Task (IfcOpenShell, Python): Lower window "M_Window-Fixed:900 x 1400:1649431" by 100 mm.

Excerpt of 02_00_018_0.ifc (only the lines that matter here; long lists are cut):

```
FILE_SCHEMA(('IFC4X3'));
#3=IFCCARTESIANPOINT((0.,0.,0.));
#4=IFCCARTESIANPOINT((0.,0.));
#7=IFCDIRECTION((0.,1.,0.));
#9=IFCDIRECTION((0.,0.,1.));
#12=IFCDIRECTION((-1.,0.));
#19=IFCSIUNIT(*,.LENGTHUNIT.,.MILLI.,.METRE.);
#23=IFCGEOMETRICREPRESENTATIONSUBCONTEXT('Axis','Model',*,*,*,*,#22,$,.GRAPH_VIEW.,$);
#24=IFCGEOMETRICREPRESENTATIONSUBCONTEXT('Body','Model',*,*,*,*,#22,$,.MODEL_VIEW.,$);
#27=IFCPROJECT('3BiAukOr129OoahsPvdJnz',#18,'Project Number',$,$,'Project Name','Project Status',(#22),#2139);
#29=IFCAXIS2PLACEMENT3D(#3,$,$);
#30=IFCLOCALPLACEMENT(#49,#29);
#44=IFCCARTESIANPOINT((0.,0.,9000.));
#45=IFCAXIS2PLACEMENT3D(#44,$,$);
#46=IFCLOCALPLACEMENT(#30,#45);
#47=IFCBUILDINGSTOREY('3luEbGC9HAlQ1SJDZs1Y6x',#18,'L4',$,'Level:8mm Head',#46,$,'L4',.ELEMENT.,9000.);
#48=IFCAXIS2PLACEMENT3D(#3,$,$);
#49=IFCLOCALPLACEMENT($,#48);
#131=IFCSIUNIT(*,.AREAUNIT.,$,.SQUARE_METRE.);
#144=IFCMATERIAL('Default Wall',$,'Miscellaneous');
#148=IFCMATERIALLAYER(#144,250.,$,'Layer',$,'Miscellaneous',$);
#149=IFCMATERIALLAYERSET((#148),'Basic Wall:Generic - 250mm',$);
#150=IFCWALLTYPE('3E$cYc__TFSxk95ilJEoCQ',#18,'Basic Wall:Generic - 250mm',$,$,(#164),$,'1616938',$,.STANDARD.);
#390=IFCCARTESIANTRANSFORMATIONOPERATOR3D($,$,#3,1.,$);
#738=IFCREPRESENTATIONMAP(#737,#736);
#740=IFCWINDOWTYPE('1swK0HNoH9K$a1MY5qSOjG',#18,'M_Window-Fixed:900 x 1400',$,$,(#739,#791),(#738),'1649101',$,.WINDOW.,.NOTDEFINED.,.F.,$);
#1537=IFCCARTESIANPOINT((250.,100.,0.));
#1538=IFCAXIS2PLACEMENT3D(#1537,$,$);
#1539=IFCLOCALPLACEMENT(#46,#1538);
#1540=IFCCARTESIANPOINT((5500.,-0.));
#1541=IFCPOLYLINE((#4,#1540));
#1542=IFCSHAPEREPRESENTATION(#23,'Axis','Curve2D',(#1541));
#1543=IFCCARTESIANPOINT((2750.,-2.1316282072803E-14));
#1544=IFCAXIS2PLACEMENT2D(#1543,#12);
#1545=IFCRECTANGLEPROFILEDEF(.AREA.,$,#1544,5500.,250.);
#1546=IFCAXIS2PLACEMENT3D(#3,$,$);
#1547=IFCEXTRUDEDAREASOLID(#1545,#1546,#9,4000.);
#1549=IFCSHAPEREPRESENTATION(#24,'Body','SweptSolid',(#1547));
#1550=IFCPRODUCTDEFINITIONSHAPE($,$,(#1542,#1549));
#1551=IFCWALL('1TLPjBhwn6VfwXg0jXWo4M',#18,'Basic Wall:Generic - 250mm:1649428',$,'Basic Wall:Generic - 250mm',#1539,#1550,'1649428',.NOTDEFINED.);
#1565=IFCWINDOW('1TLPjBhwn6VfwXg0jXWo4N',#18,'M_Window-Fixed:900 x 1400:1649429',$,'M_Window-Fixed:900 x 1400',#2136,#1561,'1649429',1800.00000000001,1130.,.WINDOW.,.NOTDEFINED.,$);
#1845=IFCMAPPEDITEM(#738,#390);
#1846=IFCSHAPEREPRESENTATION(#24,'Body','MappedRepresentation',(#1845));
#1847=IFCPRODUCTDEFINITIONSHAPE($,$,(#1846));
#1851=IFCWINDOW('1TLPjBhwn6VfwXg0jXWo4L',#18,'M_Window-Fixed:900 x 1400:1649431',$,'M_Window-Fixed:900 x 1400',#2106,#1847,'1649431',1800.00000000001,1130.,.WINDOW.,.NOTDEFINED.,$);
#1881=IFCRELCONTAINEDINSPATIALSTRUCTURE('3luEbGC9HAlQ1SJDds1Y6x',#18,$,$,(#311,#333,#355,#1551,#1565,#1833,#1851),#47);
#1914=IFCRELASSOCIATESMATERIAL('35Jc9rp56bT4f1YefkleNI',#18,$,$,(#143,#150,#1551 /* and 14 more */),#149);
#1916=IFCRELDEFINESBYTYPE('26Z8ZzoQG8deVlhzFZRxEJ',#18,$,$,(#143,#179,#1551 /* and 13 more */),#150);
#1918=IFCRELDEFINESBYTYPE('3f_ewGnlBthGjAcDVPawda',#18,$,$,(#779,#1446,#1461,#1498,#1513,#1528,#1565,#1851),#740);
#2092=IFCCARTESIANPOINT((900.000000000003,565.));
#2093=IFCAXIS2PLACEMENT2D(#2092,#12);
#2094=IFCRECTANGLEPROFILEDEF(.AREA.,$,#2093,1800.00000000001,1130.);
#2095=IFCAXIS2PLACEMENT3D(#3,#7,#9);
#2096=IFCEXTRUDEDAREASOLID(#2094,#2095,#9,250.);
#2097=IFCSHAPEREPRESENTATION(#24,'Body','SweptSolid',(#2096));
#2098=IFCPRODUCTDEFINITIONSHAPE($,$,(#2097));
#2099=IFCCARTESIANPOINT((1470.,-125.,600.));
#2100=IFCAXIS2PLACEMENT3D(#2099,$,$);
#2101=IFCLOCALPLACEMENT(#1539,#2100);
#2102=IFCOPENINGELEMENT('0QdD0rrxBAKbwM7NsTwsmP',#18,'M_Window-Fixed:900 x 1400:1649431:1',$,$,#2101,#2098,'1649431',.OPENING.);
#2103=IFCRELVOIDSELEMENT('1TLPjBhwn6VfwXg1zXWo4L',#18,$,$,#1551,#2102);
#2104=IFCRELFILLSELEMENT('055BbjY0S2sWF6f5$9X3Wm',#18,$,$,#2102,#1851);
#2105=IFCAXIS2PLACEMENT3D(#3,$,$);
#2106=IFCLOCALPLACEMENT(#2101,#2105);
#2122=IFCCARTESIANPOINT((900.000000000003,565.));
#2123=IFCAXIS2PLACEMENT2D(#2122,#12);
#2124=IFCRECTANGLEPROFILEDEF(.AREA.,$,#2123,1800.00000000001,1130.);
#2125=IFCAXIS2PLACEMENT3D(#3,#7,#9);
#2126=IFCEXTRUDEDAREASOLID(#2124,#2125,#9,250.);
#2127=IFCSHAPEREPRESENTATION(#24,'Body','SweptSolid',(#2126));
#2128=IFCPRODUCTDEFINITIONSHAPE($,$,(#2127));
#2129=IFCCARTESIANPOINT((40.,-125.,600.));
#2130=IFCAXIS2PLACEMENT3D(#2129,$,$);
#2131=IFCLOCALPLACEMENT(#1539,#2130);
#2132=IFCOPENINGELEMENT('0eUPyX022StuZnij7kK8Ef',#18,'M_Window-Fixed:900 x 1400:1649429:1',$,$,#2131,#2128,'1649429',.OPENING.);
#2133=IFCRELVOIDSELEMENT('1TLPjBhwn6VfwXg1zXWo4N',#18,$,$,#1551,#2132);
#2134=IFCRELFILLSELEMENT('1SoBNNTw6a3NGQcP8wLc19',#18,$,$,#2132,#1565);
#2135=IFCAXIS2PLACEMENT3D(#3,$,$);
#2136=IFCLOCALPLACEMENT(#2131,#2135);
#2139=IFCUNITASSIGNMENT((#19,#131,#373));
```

```python
import numpy as np
import ifcopenshell
import ifcopenshell.api.geometry
import ifcopenshell.util.placement
import ifcopenshell.util.unit

model = ifcopenshell.open("02_00_018_0.ifc")
unit_scale = ifcopenshell.util.unit.calculate_unit_scale(model)

window = model.by_id(1851)
opening = window.FillsVoids[0].RelatingOpeningElement
dz = -0.1 / unit_scale

shift = np.array([0.0, 0.0, dz])
# The window is placed relative to its opening, so it follows when the opening moves.
matrix = ifcopenshell.util.placement.get_local_placement(opening.ObjectPlacement)
matrix[:3, 3] += shift
ifcopenshell.api.geometry.edit_object_placement(
    model, product=opening, matrix=matrix, is_si=False, should_transform_children=True
)

print(f"moved by {dz * unit_scale:+.3f} m")

model.write("02_00_018_0_updated.ifc")
```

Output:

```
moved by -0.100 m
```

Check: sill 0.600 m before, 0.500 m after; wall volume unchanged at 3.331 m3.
